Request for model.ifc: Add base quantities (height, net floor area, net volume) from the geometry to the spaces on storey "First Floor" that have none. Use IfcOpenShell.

First a look at what the model holds.

```python
import ifcopenshell
import ifcopenshell.util.element
import ifcopenshell.util.unit

model = ifcopenshell.open("model.ifc")
print(model.schema)
for unit_type in ("LENGTHUNIT", "AREAUNIT", "VOLUMEUNIT"):
    print(unit_type, ifcopenshell.util.unit.calculate_unit_scale(model, unit_type))
storey = next(s for s in model.by_type("IfcBuildingStorey") if s.Name == "First Floor")
spaces = [e for e in ifcopenshell.util.element.get_decomposition(storey) if e.is_a("IfcSpace")]
for e in sorted(spaces, key=lambda e: e.id()):
    print(e.id(), e.is_a(), e.Name, list(ifcopenshell.util.element.get_psets(e, qtos_only=True)), sep=" | ")
```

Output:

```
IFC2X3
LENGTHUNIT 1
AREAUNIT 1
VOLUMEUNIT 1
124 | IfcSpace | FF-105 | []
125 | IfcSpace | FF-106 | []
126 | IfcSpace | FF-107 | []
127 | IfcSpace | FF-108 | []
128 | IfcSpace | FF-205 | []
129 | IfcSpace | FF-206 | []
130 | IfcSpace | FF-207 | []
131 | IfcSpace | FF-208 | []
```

```python
import ifcopenshell
import ifcopenshell.api.pset
import ifcopenshell.geom
import ifcopenshell.util.element
import ifcopenshell.util.shape
import ifcopenshell.util.unit

model = ifcopenshell.open("model.ifc")
unit_scale = ifcopenshell.util.unit.calculate_unit_scale(model)
area_scale = ifcopenshell.util.unit.calculate_unit_scale(model, "AREAUNIT")
volume_scale = ifcopenshell.util.unit.calculate_unit_scale(model, "VOLUMEUNIT")
settings = ifcopenshell.geom.settings()

storey = next(s for s in model.by_type("IfcBuildingStorey") if s.Name == "First Floor")
spaces = [e for e in ifcopenshell.util.element.get_decomposition(storey) if e.is_a("IfcSpace")]

for e in sorted(spaces, key=lambda e: e.id()):
    if ifcopenshell.util.element.get_psets(e, qtos_only=True, should_inherit=False):
        continue
    # Geometry comes back in metres, in the element's own axes.
    shape = ifcopenshell.geom.create_shape(settings, e)
    values = {
        "Height": ifcopenshell.util.shape.get_z(shape.geometry) / unit_scale,
        "NetFloorArea": ifcopenshell.util.shape.get_footprint_area(shape.geometry) / area_scale,
        "NetVolume": ifcopenshell.util.shape.get_volume(shape.geometry) / volume_scale,
    }
    qto = ifcopenshell.api.pset.add_qto(model, product=e, name="BaseQuantities")
    ifcopenshell.api.pset.edit_qto(model, qto=qto, properties=values)
    print(e.id(), {k: round(v, 3) for k, v in values.items()})

model.write("model_v2.ifc")
```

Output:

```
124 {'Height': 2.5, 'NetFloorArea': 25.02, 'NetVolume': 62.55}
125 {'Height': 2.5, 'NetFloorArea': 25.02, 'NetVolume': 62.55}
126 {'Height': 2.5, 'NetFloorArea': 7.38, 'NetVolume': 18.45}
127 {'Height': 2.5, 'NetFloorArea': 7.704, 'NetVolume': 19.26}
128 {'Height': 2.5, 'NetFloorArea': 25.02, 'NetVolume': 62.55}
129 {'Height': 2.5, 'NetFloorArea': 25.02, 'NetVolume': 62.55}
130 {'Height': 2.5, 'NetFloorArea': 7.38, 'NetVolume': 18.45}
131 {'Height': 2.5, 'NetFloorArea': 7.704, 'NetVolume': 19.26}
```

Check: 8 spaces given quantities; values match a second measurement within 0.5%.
